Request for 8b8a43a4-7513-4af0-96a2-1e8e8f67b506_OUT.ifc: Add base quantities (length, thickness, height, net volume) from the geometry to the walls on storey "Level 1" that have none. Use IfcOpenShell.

First a look at what the model holds.

```python
import ifcopenshell
import ifcopenshell.util.element
import ifcopenshell.util.unit

model = ifcopenshell.open("8b8a43a4-7513-4af0-96a2-1e8e8f67b506_OUT.ifc")
print(model.schema)
for unit_type in ("LENGTHUNIT", "AREAUNIT", "VOLUMEUNIT"):
    print(unit_type, ifcopenshell.util.unit.calculate_unit_scale(model, unit_type))
storey = next(s for s in model.by_type("IfcBuildingStorey") if s.Name == "Level 1")
walls = [e for e in ifcopenshell.util.element.get_decomposition(storey) if e.is_a("IfcWall")]
for e in sorted(walls, key=lambda e: e.id()):
    print(e.id(), e.is_a(), e.Name, list(ifcopenshell.util.element.get_psets(e, qtos_only=True)), sep=" | ")
```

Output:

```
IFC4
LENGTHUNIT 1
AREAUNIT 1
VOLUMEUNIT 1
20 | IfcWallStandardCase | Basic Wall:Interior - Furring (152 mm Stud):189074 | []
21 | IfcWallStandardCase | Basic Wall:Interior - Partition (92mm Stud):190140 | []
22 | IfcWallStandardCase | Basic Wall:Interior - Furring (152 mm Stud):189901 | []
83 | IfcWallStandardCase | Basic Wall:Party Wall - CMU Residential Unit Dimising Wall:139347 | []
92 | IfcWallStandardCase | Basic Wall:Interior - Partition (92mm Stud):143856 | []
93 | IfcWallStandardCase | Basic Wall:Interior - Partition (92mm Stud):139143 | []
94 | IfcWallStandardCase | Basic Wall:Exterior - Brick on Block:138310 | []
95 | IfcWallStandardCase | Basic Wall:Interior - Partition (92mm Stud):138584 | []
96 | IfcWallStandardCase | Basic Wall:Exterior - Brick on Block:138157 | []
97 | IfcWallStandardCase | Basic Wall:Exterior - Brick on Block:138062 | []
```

```python
import ifcopenshell
import ifcopenshell.api.pset
import ifcopenshell.geom
import ifcopenshell.util.element
import ifcopenshell.util.shape
import ifcopenshell.util.unit

model = ifcopenshell.open("8b8a43a4-7513-4af0-96a2-1e8e8f67b506_OUT.ifc")
unit_scale = ifcopenshell.util.unit.calculate_unit_scale(model)
volume_scale = ifcopenshell.util.unit.calculate_unit_scale(model, "VOLUMEUNIT")
settings = ifcopenshell.geom.settings()

storey = next(s for s in model.by_type("IfcBuildingStorey") if s.Name == "Level 1")
walls = [e for e in ifcopenshell.util.element.get_decomposition(storey) if e.is_a("IfcWall")]

for e in sorted(walls, key=lambda e: e.id()):
    if ifcopenshell.util.element.get_psets(e, qtos_only=True, should_inherit=False):
        continue
    # Geometry comes back in metres, in the element's own axes.
    shape = ifcopenshell.geom.create_shape(settings, e)
    values = {
        "Length": ifcopenshell.util.shape.get_x(shape.geometry) / unit_scale,
        "Width": ifcopenshell.util.shape.get_y(shape.geometry) / unit_scale,
        "Height": ifcopenshell.util.shape.get_z(shape.geometry) / unit_scale,
        "NetVolume": ifcopenshell.util.shape.get_volume(shape.geometry) / volume_scale,
    }
    qto = ifcopenshell.api.pset.add_qto(model, product=e, name="Qto_WallBaseQuantities")
    ifcopenshell.api.pset.edit_qto(model, qto=qto, properties=values)
    print(e.id(), {k: round(v, 3) for k, v in values.items()})

model.write("8b8a43a4-7513-4af0-96a2-1e8e8f67b506_OUT_edited.ifc")
```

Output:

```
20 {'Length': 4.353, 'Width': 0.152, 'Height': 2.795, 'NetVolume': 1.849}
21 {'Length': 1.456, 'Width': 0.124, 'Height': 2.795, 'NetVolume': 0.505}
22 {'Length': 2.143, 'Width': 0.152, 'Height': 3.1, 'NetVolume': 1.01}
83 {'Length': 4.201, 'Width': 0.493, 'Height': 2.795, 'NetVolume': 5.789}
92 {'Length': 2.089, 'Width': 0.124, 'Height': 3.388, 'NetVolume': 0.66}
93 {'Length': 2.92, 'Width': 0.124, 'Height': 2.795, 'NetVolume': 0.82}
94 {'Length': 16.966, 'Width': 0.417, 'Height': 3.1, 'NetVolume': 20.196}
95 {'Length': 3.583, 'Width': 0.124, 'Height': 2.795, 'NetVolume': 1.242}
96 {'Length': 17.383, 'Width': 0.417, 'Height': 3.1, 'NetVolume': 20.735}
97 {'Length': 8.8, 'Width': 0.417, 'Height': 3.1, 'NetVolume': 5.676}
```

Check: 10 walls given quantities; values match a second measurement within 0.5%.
